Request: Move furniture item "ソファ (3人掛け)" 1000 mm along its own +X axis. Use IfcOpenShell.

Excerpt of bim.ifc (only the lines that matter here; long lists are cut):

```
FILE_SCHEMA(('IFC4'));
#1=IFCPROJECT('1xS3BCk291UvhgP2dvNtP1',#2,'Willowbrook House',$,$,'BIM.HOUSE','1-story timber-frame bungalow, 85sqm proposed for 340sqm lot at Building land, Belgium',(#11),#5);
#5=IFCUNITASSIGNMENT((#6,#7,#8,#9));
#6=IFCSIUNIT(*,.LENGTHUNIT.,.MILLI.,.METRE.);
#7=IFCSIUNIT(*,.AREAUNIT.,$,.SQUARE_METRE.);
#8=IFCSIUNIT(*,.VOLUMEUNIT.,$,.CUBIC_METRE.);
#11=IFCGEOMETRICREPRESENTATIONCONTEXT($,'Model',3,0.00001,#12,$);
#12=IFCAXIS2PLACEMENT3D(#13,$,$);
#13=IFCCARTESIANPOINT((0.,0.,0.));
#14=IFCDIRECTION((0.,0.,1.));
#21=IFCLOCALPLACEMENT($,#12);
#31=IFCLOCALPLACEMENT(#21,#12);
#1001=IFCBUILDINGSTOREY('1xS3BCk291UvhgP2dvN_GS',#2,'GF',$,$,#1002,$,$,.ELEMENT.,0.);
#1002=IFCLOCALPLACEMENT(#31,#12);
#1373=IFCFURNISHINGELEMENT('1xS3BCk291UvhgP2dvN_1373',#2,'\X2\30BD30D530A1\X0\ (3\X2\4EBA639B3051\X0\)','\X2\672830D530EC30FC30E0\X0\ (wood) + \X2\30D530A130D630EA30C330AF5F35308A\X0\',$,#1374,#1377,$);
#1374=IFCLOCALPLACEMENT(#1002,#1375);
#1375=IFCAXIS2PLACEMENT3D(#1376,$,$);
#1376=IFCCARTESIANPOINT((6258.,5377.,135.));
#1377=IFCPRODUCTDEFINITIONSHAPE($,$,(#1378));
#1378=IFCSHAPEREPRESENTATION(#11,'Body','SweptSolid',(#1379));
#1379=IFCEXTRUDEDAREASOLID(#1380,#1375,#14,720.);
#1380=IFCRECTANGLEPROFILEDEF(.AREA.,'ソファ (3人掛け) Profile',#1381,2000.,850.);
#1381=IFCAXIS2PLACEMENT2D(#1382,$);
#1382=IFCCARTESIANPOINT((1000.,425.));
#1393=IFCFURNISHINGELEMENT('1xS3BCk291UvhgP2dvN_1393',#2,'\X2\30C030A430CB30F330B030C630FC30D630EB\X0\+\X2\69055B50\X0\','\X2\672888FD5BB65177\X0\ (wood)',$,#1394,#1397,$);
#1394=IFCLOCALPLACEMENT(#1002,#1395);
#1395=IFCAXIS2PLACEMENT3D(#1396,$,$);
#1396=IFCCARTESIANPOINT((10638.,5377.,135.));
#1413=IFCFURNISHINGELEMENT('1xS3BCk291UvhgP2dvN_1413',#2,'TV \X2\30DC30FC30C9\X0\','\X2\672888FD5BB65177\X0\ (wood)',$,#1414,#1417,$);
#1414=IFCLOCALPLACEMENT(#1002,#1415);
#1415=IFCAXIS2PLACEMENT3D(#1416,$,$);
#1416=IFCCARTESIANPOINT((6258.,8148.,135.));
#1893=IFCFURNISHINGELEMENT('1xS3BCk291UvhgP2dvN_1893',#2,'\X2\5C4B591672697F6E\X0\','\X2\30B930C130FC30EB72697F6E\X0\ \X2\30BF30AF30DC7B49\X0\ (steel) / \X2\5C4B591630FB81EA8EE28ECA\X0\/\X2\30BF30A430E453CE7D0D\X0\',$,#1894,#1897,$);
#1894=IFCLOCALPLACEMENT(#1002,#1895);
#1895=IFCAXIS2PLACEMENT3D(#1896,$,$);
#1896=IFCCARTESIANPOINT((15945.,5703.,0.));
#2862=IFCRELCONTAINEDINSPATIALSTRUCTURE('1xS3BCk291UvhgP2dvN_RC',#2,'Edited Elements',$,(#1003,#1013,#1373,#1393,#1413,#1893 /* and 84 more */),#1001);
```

```python
import ifcopenshell
import ifcopenshell.api.geometry
import ifcopenshell.util.placement
import ifcopenshell.util.unit

model = ifcopenshell.open("bim.ifc")
unit_scale = ifcopenshell.util.unit.calculate_unit_scale(model)

item = model.by_id(1373)
matrix = ifcopenshell.util.placement.get_local_placement(item.ObjectPlacement)
matrix[:3, 3] += matrix[:3, 0] * 1 / unit_scale
ifcopenshell.api.geometry.edit_object_placement(model, product=item, matrix=matrix, is_si=False)

print(ifcopenshell.util.placement.get_local_placement(item.ObjectPlacement).round(3) + 0.0)

model.write("bim-out.ifc")
```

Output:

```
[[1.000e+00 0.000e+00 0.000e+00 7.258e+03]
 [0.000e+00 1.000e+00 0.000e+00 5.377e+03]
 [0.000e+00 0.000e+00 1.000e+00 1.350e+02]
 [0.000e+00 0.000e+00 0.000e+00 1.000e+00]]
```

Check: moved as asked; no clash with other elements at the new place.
